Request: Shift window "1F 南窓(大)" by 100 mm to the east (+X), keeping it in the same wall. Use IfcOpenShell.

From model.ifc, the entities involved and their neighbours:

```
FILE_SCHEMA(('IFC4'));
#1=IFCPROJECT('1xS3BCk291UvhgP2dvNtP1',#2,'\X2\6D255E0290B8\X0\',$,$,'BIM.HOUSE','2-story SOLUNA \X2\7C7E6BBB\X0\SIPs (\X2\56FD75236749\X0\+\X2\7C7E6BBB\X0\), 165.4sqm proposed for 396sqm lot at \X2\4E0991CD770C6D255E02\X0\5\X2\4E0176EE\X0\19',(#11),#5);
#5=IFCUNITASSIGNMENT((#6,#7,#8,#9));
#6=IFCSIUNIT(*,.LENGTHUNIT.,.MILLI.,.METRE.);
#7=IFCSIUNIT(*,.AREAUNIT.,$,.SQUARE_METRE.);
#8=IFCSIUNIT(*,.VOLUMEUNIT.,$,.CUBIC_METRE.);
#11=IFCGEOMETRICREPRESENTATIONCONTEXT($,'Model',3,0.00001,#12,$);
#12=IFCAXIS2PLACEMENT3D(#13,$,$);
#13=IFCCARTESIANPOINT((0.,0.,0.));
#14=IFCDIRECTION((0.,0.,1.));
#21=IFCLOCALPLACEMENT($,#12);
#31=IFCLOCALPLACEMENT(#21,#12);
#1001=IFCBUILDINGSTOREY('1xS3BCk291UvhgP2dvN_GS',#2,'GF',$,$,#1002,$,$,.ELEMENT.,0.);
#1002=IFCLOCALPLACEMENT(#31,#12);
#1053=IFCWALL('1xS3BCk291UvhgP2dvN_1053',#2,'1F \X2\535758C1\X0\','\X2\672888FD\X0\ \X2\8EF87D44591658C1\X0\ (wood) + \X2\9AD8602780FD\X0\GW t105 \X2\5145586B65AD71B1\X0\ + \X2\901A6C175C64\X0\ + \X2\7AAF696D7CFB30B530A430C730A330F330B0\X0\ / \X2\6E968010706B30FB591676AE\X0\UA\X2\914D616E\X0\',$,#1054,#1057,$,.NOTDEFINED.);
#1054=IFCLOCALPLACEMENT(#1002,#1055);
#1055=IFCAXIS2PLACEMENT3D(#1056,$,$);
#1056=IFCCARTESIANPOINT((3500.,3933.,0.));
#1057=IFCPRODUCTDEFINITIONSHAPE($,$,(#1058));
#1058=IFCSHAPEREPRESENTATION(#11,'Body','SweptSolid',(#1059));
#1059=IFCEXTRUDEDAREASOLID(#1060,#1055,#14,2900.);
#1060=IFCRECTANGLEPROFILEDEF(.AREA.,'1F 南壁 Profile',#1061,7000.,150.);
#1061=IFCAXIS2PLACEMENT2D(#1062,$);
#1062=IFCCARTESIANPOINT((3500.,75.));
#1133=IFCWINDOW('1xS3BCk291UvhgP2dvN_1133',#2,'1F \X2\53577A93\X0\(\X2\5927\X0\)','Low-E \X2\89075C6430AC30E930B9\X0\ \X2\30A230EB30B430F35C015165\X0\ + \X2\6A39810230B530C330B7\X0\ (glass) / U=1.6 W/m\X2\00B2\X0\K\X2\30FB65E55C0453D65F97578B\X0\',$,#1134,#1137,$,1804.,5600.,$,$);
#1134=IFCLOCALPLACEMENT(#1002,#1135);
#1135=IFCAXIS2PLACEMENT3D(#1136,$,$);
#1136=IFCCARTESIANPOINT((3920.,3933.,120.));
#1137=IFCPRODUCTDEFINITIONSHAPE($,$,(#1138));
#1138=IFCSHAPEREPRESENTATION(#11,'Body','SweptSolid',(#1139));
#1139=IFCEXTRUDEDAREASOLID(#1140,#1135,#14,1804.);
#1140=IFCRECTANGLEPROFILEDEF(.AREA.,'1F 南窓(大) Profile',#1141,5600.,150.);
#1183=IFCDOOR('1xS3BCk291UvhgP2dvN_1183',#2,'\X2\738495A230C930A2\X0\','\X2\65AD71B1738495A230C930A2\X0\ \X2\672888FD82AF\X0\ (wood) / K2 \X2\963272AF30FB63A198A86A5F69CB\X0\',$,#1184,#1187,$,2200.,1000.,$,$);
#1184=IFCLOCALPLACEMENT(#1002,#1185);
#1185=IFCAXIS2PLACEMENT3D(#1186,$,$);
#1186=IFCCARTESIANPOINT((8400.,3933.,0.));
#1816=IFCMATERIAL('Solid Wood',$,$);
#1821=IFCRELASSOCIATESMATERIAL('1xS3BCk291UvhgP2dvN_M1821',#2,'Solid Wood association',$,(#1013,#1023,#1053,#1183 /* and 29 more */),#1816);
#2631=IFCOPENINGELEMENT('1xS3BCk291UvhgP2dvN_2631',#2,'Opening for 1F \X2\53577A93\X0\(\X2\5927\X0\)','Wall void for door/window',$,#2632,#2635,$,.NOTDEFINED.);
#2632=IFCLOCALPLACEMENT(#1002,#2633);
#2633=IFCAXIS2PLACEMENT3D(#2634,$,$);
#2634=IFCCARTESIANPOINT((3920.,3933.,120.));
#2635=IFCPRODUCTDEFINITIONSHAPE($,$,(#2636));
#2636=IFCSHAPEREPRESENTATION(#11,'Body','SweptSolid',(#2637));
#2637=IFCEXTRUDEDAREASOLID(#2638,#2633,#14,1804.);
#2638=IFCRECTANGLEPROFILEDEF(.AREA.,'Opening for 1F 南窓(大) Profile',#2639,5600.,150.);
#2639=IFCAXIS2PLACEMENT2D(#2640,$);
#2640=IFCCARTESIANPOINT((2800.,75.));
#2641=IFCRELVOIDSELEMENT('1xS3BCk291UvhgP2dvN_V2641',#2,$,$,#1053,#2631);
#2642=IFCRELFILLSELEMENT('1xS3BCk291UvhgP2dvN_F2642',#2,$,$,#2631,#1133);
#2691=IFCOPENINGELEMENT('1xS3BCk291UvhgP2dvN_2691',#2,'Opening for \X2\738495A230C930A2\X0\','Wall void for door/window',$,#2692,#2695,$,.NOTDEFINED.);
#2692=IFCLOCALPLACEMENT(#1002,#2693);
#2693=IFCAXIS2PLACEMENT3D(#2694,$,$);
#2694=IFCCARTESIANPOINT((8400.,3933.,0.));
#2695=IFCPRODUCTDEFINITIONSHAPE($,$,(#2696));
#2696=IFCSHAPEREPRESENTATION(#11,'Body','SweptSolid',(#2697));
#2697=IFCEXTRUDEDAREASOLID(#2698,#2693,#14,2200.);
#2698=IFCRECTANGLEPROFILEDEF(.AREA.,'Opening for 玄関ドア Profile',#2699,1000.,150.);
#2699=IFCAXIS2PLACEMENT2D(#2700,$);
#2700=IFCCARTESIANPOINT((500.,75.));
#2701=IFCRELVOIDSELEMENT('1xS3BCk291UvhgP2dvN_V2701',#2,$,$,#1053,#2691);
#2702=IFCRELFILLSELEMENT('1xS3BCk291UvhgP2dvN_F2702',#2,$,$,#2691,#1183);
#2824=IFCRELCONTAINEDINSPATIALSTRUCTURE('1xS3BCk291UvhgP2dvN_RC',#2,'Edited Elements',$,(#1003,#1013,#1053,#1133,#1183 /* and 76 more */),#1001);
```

```python
import ifcopenshell
import ifcopenshell.api.geometry
import ifcopenshell.util.placement
import ifcopenshell.util.unit

model = ifcopenshell.open("model.ifc")
unit_scale = ifcopenshell.util.unit.calculate_unit_scale(model)

window = model.by_guid("1xS3BCk291UvhgP2dvN_1133")
opening = window.FillsVoids[0].RelatingOpeningElement
wall = opening.VoidsElements[0].RelatingBuildingElement

wall_matrix = ifcopenshell.util.placement.get_local_placement(wall.ObjectPlacement)
shift = wall_matrix[:3, 0] * 0.1 / unit_scale
before = ifcopenshell.util.placement.get_local_placement(window.ObjectPlacement)[:3, 3].copy()

# The window is not placed relative to its opening, so move both.
for product in (opening, window):
    matrix = ifcopenshell.util.placement.get_local_placement(product.ObjectPlacement)
    matrix[:3, 3] += shift
    ifcopenshell.api.geometry.edit_object_placement(model, product=product, matrix=matrix, is_si=False)

after = ifcopenshell.util.placement.get_local_placement(window.ObjectPlacement)[:3, 3]
print("window moved by", (after - before).round(3) + 0.0)

model.write("model_edited.ifc")
```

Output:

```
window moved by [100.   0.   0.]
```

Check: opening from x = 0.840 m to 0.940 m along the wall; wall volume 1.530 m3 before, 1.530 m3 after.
